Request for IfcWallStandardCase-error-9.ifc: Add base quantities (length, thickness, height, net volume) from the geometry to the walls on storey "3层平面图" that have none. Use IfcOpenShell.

First a look at what the model holds.

```python
import ifcopenshell
import ifcopenshell.util.element
import ifcopenshell.util.unit

model = ifcopenshell.open("IfcWallStandardCase-error-9.ifc")
print(model.schema)
for unit_type in ("LENGTHUNIT", "AREAUNIT", "VOLUMEUNIT"):
    print(unit_type, ifcopenshell.util.unit.calculate_unit_scale(model, unit_type))
storey = next(s for s in model.by_type("IfcBuildingStorey") if s.Name == "3层平面图")
walls = [e for e in ifcopenshell.util.element.get_decomposition(storey) if e.is_a("IfcWall")]
for e in sorted(walls, key=lambda e: e.id()):
    print(e.id(), e.is_a(), e.Name, list(ifcopenshell.util.element.get_psets(e, qtos_only=True)), sep=" | ")
```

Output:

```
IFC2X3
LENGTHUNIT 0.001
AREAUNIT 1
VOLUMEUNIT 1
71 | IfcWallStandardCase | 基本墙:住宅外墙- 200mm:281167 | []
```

```python
import ifcopenshell
import ifcopenshell.api.pset
import ifcopenshell.geom
import ifcopenshell.util.element
import ifcopenshell.util.shape
import ifcopenshell.util.unit

model = ifcopenshell.open("IfcWallStandardCase-error-9.ifc")
unit_scale = ifcopenshell.util.unit.calculate_unit_scale(model)
volume_scale = ifcopenshell.util.unit.calculate_unit_scale(model, "VOLUMEUNIT")
settings = ifcopenshell.geom.settings()

storey = next(s for s in model.by_type("IfcBuildingStorey") if s.Name == "3层平面图")
walls = [e for e in ifcopenshell.util.element.get_decomposition(storey) if e.is_a("IfcWall")]

for e in sorted(walls, key=lambda e: e.id()):
    if ifcopenshell.util.element.get_psets(e, qtos_only=True, should_inherit=False):
        continue
    # Geometry comes back in metres, in the element's own axes.
    shape = ifcopenshell.geom.create_shape(settings, e)
    values = {
        "Length": ifcopenshell.util.shape.get_x(shape.geometry) / unit_scale,
        "Width": ifcopenshell.util.shape.get_y(shape.geometry) / unit_scale,
        "Height": ifcopenshell.util.shape.get_z(shape.geometry) / unit_scale,
        "NetVolume": ifcopenshell.util.shape.get_volume(shape.geometry) / volume_scale,
    }
    qto = ifcopenshell.api.pset.add_qto(model, product=e, name="BaseQuantities")
    ifcopenshell.api.pset.edit_qto(model, qto=qto, properties=values)
    print(e.id(), {k: round(v, 3) for k, v in values.items()})

model.write("IfcWallStandardCase-error-9_edited.ifc")
```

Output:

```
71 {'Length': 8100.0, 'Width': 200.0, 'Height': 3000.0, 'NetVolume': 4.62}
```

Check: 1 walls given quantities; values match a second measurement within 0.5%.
